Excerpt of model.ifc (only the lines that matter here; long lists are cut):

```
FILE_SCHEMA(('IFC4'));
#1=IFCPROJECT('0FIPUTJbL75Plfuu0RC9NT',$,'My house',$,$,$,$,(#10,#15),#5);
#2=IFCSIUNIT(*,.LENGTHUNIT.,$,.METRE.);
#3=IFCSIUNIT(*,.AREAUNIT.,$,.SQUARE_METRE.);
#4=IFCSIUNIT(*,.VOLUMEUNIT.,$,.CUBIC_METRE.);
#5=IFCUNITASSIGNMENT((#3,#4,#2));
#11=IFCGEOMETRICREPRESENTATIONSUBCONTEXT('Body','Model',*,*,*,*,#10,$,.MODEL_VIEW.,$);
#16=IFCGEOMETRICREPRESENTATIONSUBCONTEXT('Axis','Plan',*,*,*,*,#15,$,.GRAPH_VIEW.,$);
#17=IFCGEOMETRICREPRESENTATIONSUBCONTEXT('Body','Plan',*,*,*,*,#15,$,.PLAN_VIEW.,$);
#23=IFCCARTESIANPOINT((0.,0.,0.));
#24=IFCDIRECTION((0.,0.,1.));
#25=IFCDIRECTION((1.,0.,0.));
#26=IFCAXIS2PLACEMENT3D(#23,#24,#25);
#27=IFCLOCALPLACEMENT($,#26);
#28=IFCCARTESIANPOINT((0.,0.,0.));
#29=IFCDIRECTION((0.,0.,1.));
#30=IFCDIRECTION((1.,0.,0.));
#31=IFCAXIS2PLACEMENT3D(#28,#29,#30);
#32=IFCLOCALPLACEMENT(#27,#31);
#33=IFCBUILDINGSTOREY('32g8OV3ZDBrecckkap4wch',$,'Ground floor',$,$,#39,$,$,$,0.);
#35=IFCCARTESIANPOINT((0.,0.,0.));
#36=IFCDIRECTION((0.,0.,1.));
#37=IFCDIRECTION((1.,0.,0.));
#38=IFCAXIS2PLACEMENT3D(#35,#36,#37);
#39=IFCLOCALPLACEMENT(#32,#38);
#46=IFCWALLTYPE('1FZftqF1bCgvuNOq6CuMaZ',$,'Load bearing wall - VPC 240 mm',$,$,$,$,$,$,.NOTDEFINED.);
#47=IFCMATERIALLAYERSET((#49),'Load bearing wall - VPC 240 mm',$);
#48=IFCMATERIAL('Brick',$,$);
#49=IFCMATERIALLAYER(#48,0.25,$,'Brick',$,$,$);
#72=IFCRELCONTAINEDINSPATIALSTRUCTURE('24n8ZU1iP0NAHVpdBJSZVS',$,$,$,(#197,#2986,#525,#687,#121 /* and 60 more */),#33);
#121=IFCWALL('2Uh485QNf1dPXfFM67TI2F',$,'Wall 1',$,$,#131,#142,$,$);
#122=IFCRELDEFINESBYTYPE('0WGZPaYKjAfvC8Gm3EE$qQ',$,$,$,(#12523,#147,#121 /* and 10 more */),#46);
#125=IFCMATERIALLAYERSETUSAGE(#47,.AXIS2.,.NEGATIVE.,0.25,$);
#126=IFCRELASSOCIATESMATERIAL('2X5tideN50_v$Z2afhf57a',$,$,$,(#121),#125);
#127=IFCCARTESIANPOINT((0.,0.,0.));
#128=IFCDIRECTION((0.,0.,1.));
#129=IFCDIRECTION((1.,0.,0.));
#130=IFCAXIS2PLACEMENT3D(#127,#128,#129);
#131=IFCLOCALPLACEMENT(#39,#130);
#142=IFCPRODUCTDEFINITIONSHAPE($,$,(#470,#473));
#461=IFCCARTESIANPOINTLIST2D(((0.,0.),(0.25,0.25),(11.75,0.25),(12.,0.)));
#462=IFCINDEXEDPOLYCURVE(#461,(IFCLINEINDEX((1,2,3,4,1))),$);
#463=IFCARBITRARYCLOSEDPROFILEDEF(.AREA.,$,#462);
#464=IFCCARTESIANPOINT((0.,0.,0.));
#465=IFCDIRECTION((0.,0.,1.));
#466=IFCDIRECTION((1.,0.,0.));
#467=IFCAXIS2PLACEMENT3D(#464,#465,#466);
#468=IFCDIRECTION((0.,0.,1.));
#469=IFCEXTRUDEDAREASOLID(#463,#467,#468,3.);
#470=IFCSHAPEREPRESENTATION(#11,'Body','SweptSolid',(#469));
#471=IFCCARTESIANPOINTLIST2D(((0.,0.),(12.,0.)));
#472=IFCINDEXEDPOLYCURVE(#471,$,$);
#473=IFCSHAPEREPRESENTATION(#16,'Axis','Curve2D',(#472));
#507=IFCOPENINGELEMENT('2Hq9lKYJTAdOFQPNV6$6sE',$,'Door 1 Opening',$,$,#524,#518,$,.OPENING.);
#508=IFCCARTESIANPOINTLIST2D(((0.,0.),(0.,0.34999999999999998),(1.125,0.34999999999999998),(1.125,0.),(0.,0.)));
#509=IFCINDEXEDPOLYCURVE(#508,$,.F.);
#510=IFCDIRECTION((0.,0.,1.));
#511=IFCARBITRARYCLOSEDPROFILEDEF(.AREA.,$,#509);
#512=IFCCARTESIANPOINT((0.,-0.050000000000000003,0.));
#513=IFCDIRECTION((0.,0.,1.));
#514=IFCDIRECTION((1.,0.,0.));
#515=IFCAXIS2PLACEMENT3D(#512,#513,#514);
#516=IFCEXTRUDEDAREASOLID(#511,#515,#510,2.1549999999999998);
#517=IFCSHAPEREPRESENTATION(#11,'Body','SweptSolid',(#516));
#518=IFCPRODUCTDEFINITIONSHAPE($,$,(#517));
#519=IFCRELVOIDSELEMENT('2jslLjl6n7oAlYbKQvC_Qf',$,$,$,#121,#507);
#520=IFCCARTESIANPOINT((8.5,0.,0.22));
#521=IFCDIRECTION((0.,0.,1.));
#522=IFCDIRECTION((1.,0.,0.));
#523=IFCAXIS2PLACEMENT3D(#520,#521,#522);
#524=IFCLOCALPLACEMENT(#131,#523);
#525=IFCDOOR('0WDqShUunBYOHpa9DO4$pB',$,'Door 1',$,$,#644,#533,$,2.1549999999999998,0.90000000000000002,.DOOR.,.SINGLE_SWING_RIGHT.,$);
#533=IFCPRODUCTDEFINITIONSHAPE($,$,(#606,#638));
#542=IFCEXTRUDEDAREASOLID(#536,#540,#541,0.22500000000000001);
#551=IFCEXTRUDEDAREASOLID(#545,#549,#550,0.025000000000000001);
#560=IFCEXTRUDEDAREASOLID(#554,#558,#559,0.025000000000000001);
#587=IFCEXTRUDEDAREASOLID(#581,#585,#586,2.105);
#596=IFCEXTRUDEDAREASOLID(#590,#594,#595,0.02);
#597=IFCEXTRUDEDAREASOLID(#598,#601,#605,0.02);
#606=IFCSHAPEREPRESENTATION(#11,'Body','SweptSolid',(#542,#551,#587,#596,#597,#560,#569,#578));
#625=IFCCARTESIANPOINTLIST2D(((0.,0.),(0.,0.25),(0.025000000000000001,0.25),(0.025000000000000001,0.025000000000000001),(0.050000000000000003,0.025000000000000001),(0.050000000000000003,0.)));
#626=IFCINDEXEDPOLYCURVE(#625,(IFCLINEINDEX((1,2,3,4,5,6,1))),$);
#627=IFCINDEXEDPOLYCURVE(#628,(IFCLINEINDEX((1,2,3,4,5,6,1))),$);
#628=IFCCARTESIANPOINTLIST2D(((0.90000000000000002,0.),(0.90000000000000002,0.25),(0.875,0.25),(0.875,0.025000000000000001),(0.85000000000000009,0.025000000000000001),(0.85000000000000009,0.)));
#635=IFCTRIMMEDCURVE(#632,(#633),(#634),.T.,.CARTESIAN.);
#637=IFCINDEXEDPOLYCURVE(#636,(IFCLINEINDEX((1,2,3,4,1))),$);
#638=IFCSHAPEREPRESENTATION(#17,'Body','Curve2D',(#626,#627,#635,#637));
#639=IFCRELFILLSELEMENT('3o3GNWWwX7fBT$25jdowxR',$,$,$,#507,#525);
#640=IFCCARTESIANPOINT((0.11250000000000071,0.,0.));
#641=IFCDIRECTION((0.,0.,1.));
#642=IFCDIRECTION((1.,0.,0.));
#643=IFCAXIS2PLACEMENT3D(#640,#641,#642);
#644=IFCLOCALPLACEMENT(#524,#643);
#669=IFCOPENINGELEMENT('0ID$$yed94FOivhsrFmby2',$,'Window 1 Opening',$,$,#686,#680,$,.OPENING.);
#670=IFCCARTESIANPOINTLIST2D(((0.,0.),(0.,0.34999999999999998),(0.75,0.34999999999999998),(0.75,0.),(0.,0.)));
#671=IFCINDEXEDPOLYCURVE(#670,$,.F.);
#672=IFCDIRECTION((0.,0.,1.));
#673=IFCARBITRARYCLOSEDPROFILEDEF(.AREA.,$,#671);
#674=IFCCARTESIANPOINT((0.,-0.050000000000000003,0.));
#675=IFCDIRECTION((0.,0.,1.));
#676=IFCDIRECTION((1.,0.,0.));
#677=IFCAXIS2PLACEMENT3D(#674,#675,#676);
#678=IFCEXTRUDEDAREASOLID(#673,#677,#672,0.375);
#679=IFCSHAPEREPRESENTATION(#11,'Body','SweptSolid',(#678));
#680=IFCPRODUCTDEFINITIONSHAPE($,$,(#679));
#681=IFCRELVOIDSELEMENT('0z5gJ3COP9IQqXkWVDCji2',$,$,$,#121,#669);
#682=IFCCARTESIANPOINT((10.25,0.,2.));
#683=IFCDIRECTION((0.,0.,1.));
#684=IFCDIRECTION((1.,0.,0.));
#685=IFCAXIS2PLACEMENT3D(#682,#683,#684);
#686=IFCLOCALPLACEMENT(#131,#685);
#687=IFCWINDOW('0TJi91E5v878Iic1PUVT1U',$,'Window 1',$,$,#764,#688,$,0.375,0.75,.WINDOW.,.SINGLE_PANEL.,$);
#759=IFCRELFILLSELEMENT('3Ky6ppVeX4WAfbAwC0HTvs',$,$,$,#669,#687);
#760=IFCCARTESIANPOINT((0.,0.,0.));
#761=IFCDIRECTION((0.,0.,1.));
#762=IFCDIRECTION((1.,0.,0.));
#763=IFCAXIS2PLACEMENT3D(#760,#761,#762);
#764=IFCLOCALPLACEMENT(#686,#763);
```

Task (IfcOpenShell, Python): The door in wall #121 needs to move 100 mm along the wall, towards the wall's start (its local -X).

```python
import ifcopenshell
import ifcopenshell.api.geometry
import ifcopenshell.util.placement

model = ifcopenshell.open("model.ifc")

door = model.by_guid("0WDqShUunBYOHpa9DO4$pB")
opening = door.FillsVoids[0].RelatingOpeningElement
wall = opening.VoidsElements[0].RelatingBuildingElement

wall_matrix = ifcopenshell.util.placement.get_local_placement(wall.ObjectPlacement)
shift = wall_matrix[:3, 0] * -0.1
before = ifcopenshell.util.placement.get_local_placement(door.ObjectPlacement)[:3, 3].copy()

# The door is placed relative to its opening, so it follows when the opening moves.
matrix = ifcopenshell.util.placement.get_local_placement(opening.ObjectPlacement)
matrix[:3, 3] += shift
ifcopenshell.api.geometry.edit_object_placement(
    model, product=opening, matrix=matrix, is_si=False, should_transform_children=True
)

after = ifcopenshell.util.placement.get_local_placement(door.ObjectPlacement)[:3, 3]
print("door moved by", (after - before).round(3) + 0.0)

model.write("model-out.ifc")
```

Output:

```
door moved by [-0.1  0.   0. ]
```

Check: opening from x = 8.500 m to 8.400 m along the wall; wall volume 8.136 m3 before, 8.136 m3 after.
